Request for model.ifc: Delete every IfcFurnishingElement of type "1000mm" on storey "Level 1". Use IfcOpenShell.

First a look at what the model holds.

```python
import ifcopenshell
import ifcopenshell.util.element

model = ifcopenshell.open("model.ifc")
print(model.schema)
storey = next(s for s in model.by_type("IfcBuildingStorey") if s.Name == "Level 1")
furniture = [e for e in ifcopenshell.util.element.get_decomposition(storey) if e.is_a("IfcFurnishingElement")]
seen = {}
for e in furniture:
    element_type = ifcopenshell.util.element.get_type(e)
    name = element_type.Name if element_type not in (None, e) else None
    seen[name] = seen.get(name, 0) + 1
for name, count in sorted(seen.items(), key=str):
    print(count, "x", name)
```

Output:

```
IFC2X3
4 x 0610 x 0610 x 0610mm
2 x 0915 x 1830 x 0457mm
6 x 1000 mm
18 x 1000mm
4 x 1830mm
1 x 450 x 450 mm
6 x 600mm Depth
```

```python
import ifcopenshell
import ifcopenshell.api.root
import ifcopenshell.util.element

model = ifcopenshell.open("model.ifc")

storey = next(s for s in model.by_type("IfcBuildingStorey") if s.Name == "Level 1")
furniture = [e for e in ifcopenshell.util.element.get_decomposition(storey) if e.is_a("IfcFurnishingElement")]
targets = [e for e in furniture if (t := ifcopenshell.util.element.get_type(e)) not in (None, e) and t.Name == "1000mm"]

for e in targets:
    ifcopenshell.api.root.remove_product(model, product=e)
print(len(targets), "removed")

model.write("model_rev.ifc")
```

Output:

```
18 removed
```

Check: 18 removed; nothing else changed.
